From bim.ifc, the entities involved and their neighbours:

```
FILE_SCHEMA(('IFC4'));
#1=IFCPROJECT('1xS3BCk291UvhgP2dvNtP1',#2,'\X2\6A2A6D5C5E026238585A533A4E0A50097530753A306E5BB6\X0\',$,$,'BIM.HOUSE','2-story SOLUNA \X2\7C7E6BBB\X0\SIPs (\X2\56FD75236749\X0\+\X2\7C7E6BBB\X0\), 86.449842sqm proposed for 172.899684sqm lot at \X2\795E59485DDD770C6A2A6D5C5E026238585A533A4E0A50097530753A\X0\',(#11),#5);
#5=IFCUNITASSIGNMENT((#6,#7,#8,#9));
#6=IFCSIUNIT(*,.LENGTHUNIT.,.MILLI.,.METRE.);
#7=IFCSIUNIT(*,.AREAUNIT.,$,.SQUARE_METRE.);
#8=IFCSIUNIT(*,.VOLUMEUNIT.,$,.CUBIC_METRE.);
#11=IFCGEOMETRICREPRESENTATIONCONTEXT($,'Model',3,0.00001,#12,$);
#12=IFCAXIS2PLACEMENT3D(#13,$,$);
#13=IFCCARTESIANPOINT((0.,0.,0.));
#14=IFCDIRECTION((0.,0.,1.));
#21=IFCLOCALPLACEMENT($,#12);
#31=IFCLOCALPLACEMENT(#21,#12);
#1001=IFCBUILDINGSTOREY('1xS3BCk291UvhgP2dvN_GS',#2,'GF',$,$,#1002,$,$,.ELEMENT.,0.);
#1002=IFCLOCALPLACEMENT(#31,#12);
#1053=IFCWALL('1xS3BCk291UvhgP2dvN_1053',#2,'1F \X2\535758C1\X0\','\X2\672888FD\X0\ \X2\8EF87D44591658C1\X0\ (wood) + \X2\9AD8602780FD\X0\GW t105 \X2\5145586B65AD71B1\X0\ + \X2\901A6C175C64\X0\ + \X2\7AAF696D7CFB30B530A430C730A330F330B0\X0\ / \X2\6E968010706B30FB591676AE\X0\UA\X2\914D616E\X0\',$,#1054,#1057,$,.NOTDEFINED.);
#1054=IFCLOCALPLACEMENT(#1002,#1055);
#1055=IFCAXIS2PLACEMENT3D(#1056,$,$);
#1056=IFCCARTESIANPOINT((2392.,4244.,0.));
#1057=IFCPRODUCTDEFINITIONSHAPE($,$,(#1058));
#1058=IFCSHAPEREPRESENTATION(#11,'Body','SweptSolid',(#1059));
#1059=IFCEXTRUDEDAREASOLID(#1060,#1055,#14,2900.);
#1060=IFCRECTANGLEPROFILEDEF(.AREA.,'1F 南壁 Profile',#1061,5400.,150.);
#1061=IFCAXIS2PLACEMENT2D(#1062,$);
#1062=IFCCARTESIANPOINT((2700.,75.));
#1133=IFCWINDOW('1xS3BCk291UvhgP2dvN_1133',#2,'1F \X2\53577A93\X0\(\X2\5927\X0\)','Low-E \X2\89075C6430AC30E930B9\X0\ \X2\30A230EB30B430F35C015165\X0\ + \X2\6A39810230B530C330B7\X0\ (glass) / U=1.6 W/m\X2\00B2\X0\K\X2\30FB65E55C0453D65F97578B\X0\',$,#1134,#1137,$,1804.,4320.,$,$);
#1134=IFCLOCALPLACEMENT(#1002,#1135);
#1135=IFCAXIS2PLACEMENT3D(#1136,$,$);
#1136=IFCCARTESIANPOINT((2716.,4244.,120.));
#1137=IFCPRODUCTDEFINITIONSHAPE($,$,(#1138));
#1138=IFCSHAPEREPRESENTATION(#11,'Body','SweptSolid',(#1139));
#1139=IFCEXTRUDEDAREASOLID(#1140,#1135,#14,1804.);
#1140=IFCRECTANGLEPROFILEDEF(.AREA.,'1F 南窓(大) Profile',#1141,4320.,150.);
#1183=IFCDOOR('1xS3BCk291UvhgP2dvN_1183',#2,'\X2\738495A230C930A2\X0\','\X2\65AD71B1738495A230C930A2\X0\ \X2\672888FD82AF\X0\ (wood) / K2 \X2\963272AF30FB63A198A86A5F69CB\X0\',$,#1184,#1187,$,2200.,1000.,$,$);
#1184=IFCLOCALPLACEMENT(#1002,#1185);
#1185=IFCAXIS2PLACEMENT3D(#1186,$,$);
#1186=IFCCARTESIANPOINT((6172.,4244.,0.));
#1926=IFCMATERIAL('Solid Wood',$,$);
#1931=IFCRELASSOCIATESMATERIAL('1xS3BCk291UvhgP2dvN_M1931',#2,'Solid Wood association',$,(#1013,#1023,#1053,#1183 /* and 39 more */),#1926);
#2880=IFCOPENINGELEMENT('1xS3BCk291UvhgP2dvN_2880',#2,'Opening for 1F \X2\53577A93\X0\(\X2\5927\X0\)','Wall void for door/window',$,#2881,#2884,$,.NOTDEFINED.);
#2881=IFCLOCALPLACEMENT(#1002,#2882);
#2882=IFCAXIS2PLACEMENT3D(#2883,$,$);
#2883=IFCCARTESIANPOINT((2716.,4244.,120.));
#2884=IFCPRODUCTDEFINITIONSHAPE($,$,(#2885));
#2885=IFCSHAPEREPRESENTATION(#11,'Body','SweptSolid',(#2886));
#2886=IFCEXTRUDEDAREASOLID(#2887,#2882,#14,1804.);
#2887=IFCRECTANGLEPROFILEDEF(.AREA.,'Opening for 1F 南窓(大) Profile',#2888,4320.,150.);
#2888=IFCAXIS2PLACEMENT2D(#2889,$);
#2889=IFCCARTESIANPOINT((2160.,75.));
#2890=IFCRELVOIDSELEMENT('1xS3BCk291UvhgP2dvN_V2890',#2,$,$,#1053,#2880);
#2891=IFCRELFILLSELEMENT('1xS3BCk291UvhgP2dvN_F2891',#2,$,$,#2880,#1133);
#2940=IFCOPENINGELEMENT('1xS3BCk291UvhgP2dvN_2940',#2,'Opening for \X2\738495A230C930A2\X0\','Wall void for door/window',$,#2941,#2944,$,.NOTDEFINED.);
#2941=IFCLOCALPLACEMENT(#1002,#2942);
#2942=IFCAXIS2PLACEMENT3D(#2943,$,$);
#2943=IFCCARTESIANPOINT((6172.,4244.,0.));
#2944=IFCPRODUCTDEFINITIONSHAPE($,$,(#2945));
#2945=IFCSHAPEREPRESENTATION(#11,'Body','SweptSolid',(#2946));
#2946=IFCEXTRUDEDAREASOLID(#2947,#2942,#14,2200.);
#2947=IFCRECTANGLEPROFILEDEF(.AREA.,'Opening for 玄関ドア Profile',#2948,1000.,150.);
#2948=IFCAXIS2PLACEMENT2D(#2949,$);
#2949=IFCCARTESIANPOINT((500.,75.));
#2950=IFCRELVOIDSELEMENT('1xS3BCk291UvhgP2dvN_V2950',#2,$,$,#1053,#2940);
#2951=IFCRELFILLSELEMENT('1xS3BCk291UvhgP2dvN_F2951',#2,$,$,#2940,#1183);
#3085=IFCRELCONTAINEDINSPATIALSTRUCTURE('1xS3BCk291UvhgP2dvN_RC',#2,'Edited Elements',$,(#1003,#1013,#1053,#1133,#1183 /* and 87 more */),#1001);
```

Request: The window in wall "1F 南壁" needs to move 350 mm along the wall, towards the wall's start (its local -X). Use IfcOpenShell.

```python
import ifcopenshell
import ifcopenshell.api.geometry
import ifcopenshell.util.placement

model = ifcopenshell.open("bim.ifc")

window = model.by_guid("1xS3BCk291UvhgP2dvN_1133")
opening = window.FillsVoids[0].RelatingOpeningElement
wall = opening.VoidsElements[0].RelatingBuildingElement

wall_matrix = ifcopenshell.util.placement.get_local_placement(wall.ObjectPlacement)
shift = wall_matrix[:3, 0] * -350.0
before = ifcopenshell.util.placement.get_local_placement(window.ObjectPlacement)[:3, 3].copy()

# The window is not placed relative to its opening, so move both.
for product in (opening, window):
    matrix = ifcopenshell.util.placement.get_local_placement(product.ObjectPlacement)
    matrix[:3, 3] += shift
    ifcopenshell.api.geometry.edit_object_placement(model, product=product, matrix=matrix, is_si=False)

after = ifcopenshell.util.placement.get_local_placement(window.ObjectPlacement)[:3, 3]
print("window moved by", (after - before).round(3) + 0.0)

model.write("bim_edited.ifc")
```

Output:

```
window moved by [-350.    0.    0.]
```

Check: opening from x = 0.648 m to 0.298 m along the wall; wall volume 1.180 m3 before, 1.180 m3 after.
